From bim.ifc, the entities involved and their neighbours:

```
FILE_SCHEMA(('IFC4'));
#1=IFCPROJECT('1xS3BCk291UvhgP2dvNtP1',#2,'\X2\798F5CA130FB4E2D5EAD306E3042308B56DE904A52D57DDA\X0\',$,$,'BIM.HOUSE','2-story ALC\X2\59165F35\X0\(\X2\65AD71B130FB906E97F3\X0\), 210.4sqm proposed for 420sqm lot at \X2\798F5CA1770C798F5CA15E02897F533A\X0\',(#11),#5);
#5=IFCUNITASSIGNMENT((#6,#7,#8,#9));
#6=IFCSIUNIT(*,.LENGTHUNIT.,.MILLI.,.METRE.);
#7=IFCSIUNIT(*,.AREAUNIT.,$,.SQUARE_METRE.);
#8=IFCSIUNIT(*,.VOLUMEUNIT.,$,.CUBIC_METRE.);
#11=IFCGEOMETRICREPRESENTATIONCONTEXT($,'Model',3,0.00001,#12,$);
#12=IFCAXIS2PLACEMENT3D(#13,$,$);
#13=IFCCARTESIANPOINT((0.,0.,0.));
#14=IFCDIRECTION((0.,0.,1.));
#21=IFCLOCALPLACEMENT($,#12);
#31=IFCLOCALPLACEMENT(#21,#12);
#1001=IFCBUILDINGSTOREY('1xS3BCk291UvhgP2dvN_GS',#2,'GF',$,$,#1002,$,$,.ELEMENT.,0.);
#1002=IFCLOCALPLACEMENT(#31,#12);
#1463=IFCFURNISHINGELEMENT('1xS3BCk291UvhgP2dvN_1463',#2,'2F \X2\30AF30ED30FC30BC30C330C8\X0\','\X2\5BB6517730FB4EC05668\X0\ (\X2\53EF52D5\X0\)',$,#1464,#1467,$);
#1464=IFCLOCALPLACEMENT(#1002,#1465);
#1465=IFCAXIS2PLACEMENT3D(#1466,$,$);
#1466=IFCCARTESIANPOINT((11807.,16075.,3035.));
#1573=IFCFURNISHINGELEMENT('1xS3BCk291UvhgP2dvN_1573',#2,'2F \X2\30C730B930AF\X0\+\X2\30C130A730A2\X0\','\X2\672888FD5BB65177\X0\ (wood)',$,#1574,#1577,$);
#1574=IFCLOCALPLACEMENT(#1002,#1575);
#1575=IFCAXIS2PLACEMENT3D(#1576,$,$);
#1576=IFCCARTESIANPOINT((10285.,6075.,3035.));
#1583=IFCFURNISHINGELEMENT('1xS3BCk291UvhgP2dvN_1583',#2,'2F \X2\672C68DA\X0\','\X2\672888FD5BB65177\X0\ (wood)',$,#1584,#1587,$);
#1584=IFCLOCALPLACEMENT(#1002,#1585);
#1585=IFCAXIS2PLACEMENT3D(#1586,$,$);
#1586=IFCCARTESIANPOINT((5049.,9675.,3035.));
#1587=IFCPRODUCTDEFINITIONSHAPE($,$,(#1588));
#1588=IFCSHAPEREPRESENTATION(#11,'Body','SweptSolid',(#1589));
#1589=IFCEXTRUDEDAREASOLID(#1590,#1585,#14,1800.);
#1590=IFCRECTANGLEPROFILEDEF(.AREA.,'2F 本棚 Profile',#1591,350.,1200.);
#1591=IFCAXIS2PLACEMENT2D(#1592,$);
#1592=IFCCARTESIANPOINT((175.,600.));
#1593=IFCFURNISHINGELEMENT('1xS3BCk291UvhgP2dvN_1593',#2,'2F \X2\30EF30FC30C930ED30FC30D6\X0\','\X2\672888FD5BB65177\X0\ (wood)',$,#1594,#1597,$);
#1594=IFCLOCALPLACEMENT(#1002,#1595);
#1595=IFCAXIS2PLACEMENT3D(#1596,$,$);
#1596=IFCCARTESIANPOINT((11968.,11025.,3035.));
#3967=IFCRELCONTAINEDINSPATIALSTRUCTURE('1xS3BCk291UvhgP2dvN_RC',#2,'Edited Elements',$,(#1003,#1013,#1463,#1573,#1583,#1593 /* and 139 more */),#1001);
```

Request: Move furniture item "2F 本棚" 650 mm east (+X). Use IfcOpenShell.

```python
import ifcopenshell
import ifcopenshell.api.geometry
import ifcopenshell.util.placement
import ifcopenshell.util.unit

model = ifcopenshell.open("bim.ifc")
unit_scale = ifcopenshell.util.unit.calculate_unit_scale(model)

item = model.by_guid("1xS3BCk291UvhgP2dvN_1583")
matrix = ifcopenshell.util.placement.get_local_placement(item.ObjectPlacement)
matrix[0, 3] += 0.65 / unit_scale
ifcopenshell.api.geometry.edit_object_placement(model, product=item, matrix=matrix, is_si=False)

print(ifcopenshell.util.placement.get_local_placement(item.ObjectPlacement).round(3) + 0.0)

model.write("bim_updated.ifc")
```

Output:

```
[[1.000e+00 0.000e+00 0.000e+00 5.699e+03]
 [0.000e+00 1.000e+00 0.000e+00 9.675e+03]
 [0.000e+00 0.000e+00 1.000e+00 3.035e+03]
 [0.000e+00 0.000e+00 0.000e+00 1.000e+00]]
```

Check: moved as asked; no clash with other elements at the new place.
